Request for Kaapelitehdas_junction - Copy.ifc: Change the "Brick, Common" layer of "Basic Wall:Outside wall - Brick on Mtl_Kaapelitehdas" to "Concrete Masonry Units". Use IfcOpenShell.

First a look at what the model holds.

```python
import ifcopenshell
import ifcopenshell.util.element

model = ifcopenshell.open("Kaapelitehdas_junction - Copy.ifc")
print(model.schema)
for layer_set in model.by_type("IfcMaterialLayerSet"):
    if layer_set.LayerSetName == "Basic Wall:Outside wall - Brick on Mtl_Kaapelitehdas":
        for layer in layer_set.MaterialLayers:
            print(layer.id(), layer.Material and layer.Material.Name, layer.LayerThickness, sep=" | ")
        print(len(ifcopenshell.util.element.get_elements_by_material(model, layer_set)), "elements and types use it")
print(sorted(m.Name for m in model.by_type("IfcMaterial") if m.Name)[:60])
```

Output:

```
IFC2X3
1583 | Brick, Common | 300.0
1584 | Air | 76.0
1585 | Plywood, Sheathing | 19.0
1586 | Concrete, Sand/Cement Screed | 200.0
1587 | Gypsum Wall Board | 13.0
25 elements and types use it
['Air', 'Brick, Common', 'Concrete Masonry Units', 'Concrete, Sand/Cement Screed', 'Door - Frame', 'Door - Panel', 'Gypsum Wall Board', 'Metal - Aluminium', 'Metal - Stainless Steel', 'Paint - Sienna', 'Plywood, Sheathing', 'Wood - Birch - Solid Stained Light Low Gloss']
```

```python
import ifcopenshell
import ifcopenshell.api.material

model = ifcopenshell.open("Kaapelitehdas_junction - Copy.ifc")

layer_set = next(s for s in model.by_type("IfcMaterialLayerSet") if s.LayerSetName == "Basic Wall:Outside wall - Brick on Mtl_Kaapelitehdas")
layer = next(l for l in layer_set.MaterialLayers if l.Material and l.Material.Name == "Brick, Common")
material = next(m for m in model.by_type("IfcMaterial") if m.Name == "Concrete Masonry Units")

# Point this one layer at the other material; renaming the old one would change it everywhere.
ifcopenshell.api.material.edit_layer(model, layer=layer, attributes={}, material=material)

print([l.Material.Name if l.Material else None for l in layer_set.MaterialLayers])

model.write("Kaapelitehdas_junction - Copy_v2.ifc")
```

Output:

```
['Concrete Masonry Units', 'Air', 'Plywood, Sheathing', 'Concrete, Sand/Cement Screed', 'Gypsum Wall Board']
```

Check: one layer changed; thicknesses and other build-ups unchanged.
